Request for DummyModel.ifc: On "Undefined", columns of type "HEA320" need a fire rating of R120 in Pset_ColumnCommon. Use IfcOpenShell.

First a look at what the model holds.

```python
import ifcopenshell
import ifcopenshell.util.element

model = ifcopenshell.open("DummyModel.ifc")
print(model.schema)
storey = next(s for s in model.by_type("IfcBuildingStorey") if s.Name == "Undefined")
columns = [e for e in ifcopenshell.util.element.get_decomposition(storey) if e.is_a("IfcColumn")]
seen = {}
for e in columns:
    element_type = ifcopenshell.util.element.get_type(e)
    key = (element_type.Name if element_type != e and element_type else None, ifcopenshell.util.element.get_pset(e, "Pset_ColumnCommon", "FireRating"))
    seen[key] = seen.get(key, 0) + 1
for (name, value), count in sorted(seen.items(), key=str):
    print(count, "x", name, "|", value)
```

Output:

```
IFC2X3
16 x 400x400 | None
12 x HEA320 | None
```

```python
import ifcopenshell
import ifcopenshell.api.pset
import ifcopenshell.util.element

model = ifcopenshell.open("DummyModel.ifc")

storey = next(s for s in model.by_type("IfcBuildingStorey") if s.Name == "Undefined")
columns = [e for e in ifcopenshell.util.element.get_decomposition(storey) if e.is_a("IfcColumn")]

count = 0
for e in columns:
    element_type = ifcopenshell.util.element.get_type(e)
    if element_type in (None, e) or element_type.Name != "HEA320":
        continue
    found = ifcopenshell.util.element.get_pset(e, "Pset_ColumnCommon", should_inherit=False)
    if found:
        pset = model.by_id(found["id"])
        if len(ifcopenshell.util.element.get_elements_by_pset(pset)) > 1:
            pset = ifcopenshell.api.pset.unshare_pset(model, products=[e], pset=pset)[0]
    else:
        pset = ifcopenshell.api.pset.add_pset(model, product=e, name="Pset_ColumnCommon")
    ifcopenshell.api.pset.edit_pset(model, pset=pset, properties={"FireRating": "R120"})
    count += 1

print(count, "columns updated")

model.write("DummyModel_edited.ifc")
```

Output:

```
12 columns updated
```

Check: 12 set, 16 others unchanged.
